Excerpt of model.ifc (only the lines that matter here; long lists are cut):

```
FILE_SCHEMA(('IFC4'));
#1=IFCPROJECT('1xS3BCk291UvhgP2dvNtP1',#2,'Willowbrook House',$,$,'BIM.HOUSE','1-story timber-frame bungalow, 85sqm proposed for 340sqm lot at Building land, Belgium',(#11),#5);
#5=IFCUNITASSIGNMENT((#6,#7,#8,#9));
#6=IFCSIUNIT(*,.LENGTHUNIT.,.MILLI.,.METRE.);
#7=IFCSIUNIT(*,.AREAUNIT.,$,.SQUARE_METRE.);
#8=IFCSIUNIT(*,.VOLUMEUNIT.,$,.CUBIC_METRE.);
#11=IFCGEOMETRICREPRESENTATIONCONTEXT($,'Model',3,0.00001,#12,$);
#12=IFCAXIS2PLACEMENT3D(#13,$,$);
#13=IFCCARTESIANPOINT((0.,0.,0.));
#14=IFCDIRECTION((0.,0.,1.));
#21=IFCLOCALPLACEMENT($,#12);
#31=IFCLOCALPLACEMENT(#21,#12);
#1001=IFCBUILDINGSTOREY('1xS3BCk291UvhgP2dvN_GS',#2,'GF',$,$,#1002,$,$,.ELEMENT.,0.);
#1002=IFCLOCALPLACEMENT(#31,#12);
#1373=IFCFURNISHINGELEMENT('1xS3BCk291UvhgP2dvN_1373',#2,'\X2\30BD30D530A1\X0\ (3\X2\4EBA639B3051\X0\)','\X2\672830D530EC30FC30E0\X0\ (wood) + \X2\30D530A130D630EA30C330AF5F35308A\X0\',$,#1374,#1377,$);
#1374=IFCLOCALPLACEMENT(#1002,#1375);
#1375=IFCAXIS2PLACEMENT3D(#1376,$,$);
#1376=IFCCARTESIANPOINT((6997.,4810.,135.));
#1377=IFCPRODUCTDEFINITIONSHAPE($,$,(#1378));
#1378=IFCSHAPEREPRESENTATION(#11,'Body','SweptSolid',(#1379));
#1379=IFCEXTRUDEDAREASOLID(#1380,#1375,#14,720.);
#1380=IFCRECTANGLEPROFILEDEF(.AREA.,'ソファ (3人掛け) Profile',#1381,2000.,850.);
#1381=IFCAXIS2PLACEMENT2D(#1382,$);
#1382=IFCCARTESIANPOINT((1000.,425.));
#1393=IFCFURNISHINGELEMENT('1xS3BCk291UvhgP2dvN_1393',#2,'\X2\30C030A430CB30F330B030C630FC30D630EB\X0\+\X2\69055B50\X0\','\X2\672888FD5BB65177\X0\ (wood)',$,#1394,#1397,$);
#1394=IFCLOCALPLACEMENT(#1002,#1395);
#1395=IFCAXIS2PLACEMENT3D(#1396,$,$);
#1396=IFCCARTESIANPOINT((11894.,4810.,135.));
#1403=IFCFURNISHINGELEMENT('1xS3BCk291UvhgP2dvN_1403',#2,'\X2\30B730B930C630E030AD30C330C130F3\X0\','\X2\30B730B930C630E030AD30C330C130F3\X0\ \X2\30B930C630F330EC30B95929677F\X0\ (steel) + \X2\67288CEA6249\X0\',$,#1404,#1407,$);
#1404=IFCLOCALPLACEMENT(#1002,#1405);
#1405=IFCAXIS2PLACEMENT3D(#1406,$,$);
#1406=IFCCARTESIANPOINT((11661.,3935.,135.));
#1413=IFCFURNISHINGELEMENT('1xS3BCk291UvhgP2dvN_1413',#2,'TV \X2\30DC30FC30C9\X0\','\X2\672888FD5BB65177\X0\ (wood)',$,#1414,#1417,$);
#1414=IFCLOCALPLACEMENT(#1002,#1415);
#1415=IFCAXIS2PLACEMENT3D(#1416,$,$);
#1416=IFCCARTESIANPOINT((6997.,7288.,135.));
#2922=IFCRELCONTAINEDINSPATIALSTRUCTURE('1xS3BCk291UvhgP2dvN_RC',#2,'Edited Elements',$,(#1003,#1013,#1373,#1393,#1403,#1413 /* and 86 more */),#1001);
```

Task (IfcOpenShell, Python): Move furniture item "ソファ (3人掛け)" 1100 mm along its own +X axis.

```python
import ifcopenshell
import ifcopenshell.api.geometry
import ifcopenshell.util.placement

model = ifcopenshell.open("model.ifc")

item = model.by_guid("1xS3BCk291UvhgP2dvN_1373")
matrix = ifcopenshell.util.placement.get_local_placement(item.ObjectPlacement)
matrix[:3, 3] += matrix[:3, 0] * 1100.0
ifcopenshell.api.geometry.edit_object_placement(model, product=item, matrix=matrix, is_si=False)

print(ifcopenshell.util.placement.get_local_placement(item.ObjectPlacement).round(3) + 0.0)

model.write("model_v2.ifc")
```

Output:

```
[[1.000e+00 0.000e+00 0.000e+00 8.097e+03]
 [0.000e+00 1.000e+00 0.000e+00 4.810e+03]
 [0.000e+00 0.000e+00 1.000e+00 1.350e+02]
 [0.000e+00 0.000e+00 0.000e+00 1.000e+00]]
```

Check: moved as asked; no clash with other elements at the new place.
